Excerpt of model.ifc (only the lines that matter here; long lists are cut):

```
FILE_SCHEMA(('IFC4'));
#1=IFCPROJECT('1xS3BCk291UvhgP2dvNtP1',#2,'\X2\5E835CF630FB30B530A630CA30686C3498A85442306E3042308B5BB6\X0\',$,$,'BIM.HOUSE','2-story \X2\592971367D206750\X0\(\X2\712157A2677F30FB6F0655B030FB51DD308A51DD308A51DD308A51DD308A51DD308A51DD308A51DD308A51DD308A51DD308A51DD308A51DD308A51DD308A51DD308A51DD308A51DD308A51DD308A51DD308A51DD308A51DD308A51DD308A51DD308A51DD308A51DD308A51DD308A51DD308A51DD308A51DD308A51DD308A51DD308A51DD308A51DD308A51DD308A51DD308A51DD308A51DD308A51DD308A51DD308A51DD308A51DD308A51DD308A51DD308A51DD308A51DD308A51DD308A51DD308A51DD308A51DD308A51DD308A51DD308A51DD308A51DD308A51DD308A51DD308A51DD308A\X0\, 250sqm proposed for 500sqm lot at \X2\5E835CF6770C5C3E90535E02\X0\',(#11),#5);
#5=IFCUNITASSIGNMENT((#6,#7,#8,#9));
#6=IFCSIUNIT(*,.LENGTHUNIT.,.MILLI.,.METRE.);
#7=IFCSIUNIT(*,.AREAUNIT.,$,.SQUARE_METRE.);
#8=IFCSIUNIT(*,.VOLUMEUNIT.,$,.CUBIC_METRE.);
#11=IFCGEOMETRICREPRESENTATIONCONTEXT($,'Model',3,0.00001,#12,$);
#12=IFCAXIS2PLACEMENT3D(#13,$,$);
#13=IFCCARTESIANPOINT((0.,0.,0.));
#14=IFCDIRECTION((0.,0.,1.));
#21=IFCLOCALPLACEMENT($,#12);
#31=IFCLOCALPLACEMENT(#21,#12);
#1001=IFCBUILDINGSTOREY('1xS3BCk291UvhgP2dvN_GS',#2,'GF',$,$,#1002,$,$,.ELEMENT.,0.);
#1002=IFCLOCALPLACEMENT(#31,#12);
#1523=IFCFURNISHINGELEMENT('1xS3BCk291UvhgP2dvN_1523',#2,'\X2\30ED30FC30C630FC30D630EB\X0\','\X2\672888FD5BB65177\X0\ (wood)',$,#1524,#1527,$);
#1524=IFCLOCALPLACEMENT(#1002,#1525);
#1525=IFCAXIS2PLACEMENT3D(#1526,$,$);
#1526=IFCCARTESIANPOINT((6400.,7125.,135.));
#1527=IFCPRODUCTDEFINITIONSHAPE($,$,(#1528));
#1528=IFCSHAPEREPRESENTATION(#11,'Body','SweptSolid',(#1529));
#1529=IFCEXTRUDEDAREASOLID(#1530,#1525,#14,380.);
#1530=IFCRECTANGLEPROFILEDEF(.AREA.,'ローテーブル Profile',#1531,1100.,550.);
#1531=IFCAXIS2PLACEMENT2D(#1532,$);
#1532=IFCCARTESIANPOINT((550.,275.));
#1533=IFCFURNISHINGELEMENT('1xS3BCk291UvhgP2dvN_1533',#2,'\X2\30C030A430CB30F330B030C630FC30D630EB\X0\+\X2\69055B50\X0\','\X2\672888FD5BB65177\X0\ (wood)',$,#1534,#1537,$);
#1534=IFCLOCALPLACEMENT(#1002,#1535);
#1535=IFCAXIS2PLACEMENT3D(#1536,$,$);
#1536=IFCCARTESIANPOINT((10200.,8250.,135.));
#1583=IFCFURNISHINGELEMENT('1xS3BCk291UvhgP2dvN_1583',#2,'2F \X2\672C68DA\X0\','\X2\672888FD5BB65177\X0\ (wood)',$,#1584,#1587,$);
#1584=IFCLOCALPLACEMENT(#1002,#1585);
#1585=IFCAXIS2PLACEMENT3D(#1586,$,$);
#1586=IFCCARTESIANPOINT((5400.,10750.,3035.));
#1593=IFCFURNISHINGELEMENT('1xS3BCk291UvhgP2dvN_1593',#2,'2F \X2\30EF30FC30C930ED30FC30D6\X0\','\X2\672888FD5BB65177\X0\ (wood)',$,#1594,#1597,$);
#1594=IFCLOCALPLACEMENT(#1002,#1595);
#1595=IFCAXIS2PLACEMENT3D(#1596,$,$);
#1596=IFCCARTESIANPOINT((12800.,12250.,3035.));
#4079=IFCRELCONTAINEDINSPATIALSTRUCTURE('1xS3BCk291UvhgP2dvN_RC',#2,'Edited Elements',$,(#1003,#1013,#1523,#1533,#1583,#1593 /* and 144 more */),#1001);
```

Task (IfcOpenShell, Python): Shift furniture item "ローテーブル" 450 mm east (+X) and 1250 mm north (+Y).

```python
import ifcopenshell
import ifcopenshell.api.geometry
import ifcopenshell.util.placement
import ifcopenshell.util.unit

model = ifcopenshell.open("model.ifc")
unit_scale = ifcopenshell.util.unit.calculate_unit_scale(model)

item = model.by_guid("1xS3BCk291UvhgP2dvN_1523")
matrix = ifcopenshell.util.placement.get_local_placement(item.ObjectPlacement)
matrix[0, 3] += 0.45 / unit_scale
matrix[1, 3] += 1.25 / unit_scale
ifcopenshell.api.geometry.edit_object_placement(model, product=item, matrix=matrix, is_si=False)

print(ifcopenshell.util.placement.get_local_placement(item.ObjectPlacement).round(3) + 0.0)

model.write("model_rev.ifc")
```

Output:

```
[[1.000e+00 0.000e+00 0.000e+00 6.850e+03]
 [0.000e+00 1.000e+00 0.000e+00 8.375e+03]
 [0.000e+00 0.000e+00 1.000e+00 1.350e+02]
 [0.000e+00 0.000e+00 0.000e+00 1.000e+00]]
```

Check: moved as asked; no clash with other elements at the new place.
